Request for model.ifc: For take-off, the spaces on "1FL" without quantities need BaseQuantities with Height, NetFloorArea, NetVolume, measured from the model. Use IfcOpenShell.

First a look at what the model holds.

```python
import ifcopenshell
import ifcopenshell.util.element
import ifcopenshell.util.unit

model = ifcopenshell.open("model.ifc")
print(model.schema)
for unit_type in ("LENGTHUNIT", "AREAUNIT", "VOLUMEUNIT"):
    print(unit_type, ifcopenshell.util.unit.calculate_unit_scale(model, unit_type))
storey = next(s for s in model.by_type("IfcBuildingStorey") if s.Name == "1FL")
spaces = [e for e in ifcopenshell.util.element.get_decomposition(storey) if e.is_a("IfcSpace")]
for e in sorted(spaces, key=lambda e: e.id()):
    print(e.id(), e.is_a(), e.Name, list(ifcopenshell.util.element.get_psets(e, qtos_only=True)), sep=" | ")
```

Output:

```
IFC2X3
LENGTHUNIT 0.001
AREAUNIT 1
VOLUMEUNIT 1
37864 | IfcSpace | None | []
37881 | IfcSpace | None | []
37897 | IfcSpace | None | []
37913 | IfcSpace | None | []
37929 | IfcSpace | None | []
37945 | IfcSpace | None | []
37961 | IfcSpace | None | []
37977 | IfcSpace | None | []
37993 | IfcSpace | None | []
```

```python
import ifcopenshell
import ifcopenshell.api.pset
import ifcopenshell.geom
import ifcopenshell.util.element
import ifcopenshell.util.shape
import ifcopenshell.util.unit

model = ifcopenshell.open("model.ifc")
unit_scale = ifcopenshell.util.unit.calculate_unit_scale(model)
area_scale = ifcopenshell.util.unit.calculate_unit_scale(model, "AREAUNIT")
volume_scale = ifcopenshell.util.unit.calculate_unit_scale(model, "VOLUMEUNIT")
settings = ifcopenshell.geom.settings()

storey = next(s for s in model.by_type("IfcBuildingStorey") if s.Name == "1FL")
spaces = [e for e in ifcopenshell.util.element.get_decomposition(storey) if e.is_a("IfcSpace")]

for e in sorted(spaces, key=lambda e: e.id()):
    if ifcopenshell.util.element.get_psets(e, qtos_only=True, should_inherit=False):
        continue
    # Geometry comes back in metres, in the element's own axes.
    shape = ifcopenshell.geom.create_shape(settings, e)
    values = {
        "Height": ifcopenshell.util.shape.get_z(shape.geometry) / unit_scale,
        "NetFloorArea": ifcopenshell.util.shape.get_footprint_area(shape.geometry) / area_scale,
        "NetVolume": ifcopenshell.util.shape.get_volume(shape.geometry) / volume_scale,
    }
    qto = ifcopenshell.api.pset.add_qto(model, product=e, name="BaseQuantities")
    ifcopenshell.api.pset.edit_qto(model, qto=qto, properties=values)
    print(e.id(), {k: round(v, 3) for k, v in values.items()})

model.write("model-out.ifc")
```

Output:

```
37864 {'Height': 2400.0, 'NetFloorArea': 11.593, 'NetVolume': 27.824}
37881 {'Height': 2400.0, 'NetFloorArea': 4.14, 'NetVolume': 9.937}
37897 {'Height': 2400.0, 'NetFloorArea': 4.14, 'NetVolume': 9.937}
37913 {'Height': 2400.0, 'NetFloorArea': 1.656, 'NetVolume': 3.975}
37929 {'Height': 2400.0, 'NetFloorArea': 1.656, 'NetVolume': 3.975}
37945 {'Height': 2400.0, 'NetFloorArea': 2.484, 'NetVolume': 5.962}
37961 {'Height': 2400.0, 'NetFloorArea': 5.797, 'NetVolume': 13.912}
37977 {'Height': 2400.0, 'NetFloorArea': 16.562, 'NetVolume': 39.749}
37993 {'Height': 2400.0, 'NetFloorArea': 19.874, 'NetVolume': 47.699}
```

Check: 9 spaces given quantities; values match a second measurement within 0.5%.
